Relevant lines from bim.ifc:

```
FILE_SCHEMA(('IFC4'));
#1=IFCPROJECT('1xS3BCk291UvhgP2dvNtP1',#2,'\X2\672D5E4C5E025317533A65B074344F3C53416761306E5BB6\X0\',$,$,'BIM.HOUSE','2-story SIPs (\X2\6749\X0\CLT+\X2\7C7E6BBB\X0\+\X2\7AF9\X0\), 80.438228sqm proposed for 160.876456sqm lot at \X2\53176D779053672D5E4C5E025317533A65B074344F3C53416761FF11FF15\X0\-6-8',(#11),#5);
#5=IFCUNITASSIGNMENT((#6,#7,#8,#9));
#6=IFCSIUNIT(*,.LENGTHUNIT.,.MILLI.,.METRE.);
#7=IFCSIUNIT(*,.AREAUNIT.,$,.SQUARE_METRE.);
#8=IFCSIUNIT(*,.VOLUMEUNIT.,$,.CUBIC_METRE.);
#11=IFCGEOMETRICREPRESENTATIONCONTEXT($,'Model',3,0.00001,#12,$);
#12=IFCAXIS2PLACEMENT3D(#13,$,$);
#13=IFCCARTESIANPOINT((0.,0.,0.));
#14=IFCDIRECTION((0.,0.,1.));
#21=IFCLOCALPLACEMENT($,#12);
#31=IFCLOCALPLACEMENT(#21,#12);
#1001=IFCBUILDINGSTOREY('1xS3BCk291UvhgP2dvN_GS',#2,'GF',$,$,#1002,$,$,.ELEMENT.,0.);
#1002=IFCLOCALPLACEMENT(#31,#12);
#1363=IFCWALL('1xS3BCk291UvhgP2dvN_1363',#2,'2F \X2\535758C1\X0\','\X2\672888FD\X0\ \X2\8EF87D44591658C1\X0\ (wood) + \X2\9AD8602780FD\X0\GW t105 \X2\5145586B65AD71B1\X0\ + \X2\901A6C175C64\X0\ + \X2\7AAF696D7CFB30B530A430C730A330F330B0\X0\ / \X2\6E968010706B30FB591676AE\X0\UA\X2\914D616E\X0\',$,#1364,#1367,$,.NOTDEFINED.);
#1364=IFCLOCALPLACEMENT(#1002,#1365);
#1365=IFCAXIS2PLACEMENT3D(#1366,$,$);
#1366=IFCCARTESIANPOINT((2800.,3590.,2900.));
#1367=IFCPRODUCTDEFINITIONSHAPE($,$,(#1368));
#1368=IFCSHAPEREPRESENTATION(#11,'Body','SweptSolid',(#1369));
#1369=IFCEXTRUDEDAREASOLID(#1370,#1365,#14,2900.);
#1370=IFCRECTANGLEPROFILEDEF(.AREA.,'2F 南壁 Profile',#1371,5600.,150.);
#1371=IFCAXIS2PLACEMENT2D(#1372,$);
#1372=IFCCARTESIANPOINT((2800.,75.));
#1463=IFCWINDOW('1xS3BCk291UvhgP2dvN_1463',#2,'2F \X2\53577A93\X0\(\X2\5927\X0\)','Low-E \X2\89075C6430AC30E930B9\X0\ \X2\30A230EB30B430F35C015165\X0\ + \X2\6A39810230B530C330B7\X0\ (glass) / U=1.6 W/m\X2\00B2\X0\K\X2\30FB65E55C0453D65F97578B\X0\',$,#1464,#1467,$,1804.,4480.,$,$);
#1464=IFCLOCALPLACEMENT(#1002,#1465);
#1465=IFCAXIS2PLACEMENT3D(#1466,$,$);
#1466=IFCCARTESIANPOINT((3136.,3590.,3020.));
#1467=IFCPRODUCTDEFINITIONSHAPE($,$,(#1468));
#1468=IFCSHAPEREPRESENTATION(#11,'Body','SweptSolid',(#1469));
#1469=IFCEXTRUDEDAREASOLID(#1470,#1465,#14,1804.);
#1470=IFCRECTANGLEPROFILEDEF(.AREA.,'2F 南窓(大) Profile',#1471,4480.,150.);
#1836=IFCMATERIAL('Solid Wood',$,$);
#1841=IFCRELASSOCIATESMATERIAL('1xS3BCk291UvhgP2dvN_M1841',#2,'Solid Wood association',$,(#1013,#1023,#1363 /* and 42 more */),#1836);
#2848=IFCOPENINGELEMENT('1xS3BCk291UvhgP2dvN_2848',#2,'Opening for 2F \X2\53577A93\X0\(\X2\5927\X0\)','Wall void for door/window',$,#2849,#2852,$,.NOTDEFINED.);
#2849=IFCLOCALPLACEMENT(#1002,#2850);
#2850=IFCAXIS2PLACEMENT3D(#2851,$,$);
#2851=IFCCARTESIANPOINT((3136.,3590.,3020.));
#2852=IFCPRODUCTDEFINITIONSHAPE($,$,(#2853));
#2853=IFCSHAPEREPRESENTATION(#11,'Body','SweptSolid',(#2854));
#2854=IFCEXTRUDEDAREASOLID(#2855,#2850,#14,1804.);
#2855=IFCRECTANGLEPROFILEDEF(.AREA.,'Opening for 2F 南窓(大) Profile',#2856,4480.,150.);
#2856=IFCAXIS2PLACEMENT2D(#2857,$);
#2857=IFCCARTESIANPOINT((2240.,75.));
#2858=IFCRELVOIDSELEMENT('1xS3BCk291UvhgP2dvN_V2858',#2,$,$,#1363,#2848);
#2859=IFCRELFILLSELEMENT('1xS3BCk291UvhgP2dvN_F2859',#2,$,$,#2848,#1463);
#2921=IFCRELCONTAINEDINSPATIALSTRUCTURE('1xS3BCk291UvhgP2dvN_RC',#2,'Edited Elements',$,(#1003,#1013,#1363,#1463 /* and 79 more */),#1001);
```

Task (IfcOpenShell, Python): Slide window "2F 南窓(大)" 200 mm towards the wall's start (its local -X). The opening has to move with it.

```python
import ifcopenshell
import ifcopenshell.api.geometry
import ifcopenshell.util.placement

model = ifcopenshell.open("bim.ifc")

window = model.by_id(1463)
opening = window.FillsVoids[0].RelatingOpeningElement
wall = opening.VoidsElements[0].RelatingBuildingElement

wall_matrix = ifcopenshell.util.placement.get_local_placement(wall.ObjectPlacement)
shift = wall_matrix[:3, 0] * -200.0
before = ifcopenshell.util.placement.get_local_placement(window.ObjectPlacement)[:3, 3].copy()

# The window is not placed relative to its opening, so move both.
for product in (opening, window):
    matrix = ifcopenshell.util.placement.get_local_placement(product.ObjectPlacement)
    matrix[:3, 3] += shift
    ifcopenshell.api.geometry.edit_object_placement(model, product=product, matrix=matrix, is_si=False)

after = ifcopenshell.util.placement.get_local_placement(window.ObjectPlacement)[:3, 3]
print("window moved by", (after - before).round(3) + 0.0)

model.write("bim_updated.ifc")
```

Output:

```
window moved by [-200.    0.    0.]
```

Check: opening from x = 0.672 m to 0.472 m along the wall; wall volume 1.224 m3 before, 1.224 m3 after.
